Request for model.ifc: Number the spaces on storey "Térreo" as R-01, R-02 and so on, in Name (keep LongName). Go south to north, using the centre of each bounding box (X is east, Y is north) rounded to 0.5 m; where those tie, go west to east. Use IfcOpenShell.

First a look at what the model holds.

```python
import ifcopenshell
import ifcopenshell.util.element
import ifcopenshell.util.placement

model = ifcopenshell.open("model.ifc")
print(model.schema)
storey = next(s for s in model.by_type("IfcBuildingStorey") if s.Name == "Térreo")
spaces = [e for e in ifcopenshell.util.element.get_decomposition(storey) if e.is_a("IfcSpace")]
for e in sorted(spaces, key=lambda e: e.id()):
    origin = ifcopenshell.util.placement.get_local_placement(e.ObjectPlacement)[:3, 3]
    print(e.id(), e.Name, e.LongName, origin.round(2) + 0.0, sep=" | ")
```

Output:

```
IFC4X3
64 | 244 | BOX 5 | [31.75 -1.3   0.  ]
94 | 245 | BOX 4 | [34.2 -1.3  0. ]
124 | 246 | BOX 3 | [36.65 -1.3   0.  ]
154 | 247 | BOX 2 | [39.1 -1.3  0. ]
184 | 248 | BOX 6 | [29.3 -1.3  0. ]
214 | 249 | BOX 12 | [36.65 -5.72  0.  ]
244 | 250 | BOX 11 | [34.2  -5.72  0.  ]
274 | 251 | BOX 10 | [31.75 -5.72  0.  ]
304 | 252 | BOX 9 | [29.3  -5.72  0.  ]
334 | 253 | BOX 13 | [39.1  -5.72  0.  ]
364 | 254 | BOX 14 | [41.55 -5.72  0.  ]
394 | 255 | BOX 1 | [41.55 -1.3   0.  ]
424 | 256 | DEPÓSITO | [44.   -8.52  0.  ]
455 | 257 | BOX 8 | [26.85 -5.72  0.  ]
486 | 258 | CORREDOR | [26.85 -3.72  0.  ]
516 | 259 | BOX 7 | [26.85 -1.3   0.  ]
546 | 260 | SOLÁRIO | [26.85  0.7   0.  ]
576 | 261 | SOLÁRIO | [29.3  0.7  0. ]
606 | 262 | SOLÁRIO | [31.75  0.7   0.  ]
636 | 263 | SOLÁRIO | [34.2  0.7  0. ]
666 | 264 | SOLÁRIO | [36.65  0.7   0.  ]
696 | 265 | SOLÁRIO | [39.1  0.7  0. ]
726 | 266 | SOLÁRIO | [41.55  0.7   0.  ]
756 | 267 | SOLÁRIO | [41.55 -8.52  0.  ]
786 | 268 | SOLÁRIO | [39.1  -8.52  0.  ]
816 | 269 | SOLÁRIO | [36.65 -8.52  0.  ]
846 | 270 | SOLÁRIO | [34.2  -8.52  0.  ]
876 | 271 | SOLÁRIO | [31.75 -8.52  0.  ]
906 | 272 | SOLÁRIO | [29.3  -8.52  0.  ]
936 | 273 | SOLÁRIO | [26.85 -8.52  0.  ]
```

```python
import ifcopenshell
import ifcopenshell.geom
import ifcopenshell.util.element
import ifcopenshell.util.shape

model = ifcopenshell.open("model.ifc")
settings = ifcopenshell.geom.settings()
settings.set("use-world-coords", True)


def centre(element):
    shape = ifcopenshell.geom.create_shape(settings, element)
    return ifcopenshell.util.shape.get_bbox_centroid(shape.geometry)


storey = next(s for s in model.by_type("IfcBuildingStorey") if s.Name == "Térreo")
spaces = [e for e in ifcopenshell.util.element.get_decomposition(storey) if e.is_a("IfcSpace")]

# Insertion points can sit at a corner or the storey origin, so sort by the geometry (in metres).
centres = {e: centre(e) for e in spaces}
spaces.sort(key=lambda e: (round(centres[e][1] / 0.5), centres[e][0]))

for i, e in enumerate(spaces, start=1):
    number = f"R-{i:02d}"
    e.Name = number
    print(e.id(), number)

model.write("model_rev.ifc")
```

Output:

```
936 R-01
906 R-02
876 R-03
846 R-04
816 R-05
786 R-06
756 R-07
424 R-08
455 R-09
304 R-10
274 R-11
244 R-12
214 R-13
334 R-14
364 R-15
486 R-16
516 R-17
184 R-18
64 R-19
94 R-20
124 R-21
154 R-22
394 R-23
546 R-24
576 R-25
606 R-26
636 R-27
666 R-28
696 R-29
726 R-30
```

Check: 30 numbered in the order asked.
